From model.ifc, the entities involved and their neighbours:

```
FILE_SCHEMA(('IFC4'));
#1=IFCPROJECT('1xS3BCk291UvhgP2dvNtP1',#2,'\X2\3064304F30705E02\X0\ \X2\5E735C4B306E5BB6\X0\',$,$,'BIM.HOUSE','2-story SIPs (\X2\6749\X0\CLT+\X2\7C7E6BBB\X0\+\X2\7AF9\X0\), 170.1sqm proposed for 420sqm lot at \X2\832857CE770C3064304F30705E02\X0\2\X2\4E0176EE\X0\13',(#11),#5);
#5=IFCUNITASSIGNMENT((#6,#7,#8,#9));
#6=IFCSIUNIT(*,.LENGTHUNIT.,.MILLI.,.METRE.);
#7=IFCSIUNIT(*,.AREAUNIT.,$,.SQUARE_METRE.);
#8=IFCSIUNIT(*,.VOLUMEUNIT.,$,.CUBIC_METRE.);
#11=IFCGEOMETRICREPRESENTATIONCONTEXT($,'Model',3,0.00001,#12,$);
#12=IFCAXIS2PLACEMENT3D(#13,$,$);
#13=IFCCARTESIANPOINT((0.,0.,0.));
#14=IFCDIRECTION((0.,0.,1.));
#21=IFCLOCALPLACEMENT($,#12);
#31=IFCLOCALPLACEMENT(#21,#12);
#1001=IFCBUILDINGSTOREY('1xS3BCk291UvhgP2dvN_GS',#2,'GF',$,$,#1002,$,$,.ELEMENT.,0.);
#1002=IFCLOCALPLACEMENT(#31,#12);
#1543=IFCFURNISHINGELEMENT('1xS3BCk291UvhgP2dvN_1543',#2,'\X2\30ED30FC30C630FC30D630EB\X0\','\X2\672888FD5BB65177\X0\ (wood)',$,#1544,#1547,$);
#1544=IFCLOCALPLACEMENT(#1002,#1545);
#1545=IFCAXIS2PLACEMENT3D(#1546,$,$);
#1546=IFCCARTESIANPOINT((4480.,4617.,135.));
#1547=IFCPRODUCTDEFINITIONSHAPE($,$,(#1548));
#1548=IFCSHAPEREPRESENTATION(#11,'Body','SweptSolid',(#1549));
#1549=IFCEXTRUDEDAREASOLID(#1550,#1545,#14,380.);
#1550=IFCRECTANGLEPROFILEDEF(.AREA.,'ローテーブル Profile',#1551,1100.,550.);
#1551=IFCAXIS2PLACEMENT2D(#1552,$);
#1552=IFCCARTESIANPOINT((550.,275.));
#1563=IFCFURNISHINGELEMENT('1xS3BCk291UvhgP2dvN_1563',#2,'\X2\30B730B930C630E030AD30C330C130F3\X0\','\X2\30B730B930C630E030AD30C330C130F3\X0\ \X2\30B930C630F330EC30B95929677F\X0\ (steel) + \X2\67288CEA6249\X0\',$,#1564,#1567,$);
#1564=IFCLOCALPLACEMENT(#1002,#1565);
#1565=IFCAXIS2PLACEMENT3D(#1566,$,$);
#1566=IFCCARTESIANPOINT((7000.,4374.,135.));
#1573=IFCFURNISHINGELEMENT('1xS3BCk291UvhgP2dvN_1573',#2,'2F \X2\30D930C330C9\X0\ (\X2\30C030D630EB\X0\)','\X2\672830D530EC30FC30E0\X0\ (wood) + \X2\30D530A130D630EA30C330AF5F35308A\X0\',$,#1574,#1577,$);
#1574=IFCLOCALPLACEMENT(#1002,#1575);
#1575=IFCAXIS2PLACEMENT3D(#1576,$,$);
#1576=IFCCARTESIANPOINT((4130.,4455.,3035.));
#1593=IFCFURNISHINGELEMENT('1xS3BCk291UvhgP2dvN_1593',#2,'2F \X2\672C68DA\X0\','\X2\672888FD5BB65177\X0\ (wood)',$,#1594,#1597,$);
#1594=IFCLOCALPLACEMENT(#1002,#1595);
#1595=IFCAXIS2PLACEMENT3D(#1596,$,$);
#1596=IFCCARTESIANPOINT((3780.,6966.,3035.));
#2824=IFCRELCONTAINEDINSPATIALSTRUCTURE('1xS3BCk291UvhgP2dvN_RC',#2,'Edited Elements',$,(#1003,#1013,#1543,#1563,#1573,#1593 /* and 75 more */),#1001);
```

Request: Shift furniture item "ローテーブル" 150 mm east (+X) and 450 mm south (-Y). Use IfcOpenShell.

```python
import ifcopenshell
import ifcopenshell.api.geometry
import ifcopenshell.util.placement

model = ifcopenshell.open("model.ifc")

item = model.by_guid("1xS3BCk291UvhgP2dvN_1543")
matrix = ifcopenshell.util.placement.get_local_placement(item.ObjectPlacement)
matrix[0, 3] += 150.0
matrix[1, 3] -= 450.0
ifcopenshell.api.geometry.edit_object_placement(model, product=item, matrix=matrix, is_si=False)

print(ifcopenshell.util.placement.get_local_placement(item.ObjectPlacement).round(3) + 0.0)

model.write("model_v2.ifc")
```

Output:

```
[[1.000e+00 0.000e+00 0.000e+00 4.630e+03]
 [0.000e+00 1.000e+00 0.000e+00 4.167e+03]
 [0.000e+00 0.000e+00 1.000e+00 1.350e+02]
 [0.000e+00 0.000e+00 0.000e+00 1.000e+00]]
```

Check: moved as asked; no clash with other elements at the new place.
